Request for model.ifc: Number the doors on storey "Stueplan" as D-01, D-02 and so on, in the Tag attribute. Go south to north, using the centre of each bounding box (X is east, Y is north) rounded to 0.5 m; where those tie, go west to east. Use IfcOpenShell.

First a look at what the model holds.

```python
import ifcopenshell
import ifcopenshell.util.element
import ifcopenshell.util.placement

model = ifcopenshell.open("model.ifc")
print(model.schema)
storey = next(s for s in model.by_type("IfcBuildingStorey") if s.Name == "Stueplan")
doors = [e for e in ifcopenshell.util.element.get_decomposition(storey) if e.is_a("IfcDoor")]
for e in sorted(doors, key=lambda e: e.id()):
    origin = ifcopenshell.util.placement.get_local_placement(e.ObjectPlacement)[:3, 3]
    print(e.id(), e.Tag, e.Name, origin.round(2) + 0.0, sep=" | ")
```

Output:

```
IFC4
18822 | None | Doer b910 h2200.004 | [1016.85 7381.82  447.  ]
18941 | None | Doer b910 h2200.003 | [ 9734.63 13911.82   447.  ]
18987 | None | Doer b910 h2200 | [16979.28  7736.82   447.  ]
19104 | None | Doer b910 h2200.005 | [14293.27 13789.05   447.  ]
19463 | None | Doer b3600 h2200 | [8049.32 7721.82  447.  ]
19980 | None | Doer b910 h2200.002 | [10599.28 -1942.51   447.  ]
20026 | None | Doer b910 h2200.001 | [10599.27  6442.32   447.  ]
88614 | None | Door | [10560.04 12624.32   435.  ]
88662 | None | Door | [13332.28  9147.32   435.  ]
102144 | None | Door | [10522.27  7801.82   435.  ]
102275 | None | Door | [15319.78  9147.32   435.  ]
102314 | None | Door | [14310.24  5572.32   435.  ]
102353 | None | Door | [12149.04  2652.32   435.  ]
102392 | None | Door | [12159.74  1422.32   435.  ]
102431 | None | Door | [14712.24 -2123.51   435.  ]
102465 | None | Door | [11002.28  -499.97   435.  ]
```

```python
import ifcopenshell
import ifcopenshell.geom
import ifcopenshell.util.element
import ifcopenshell.util.shape

model = ifcopenshell.open("model.ifc")
settings = ifcopenshell.geom.settings()
settings.set("use-world-coords", True)


def centre(element):
    shape = ifcopenshell.geom.create_shape(settings, element)
    return ifcopenshell.util.shape.get_bbox_centroid(shape.geometry)


storey = next(s for s in model.by_type("IfcBuildingStorey") if s.Name == "Stueplan")
doors = [e for e in ifcopenshell.util.element.get_decomposition(storey) if e.is_a("IfcDoor")]

# Insertion points can sit at a corner or the storey origin, so sort by the geometry (in metres).
centres = {e: centre(e) for e in doors}
doors.sort(key=lambda e: (round(centres[e][1] / 0.5), centres[e][0]))

for i, e in enumerate(doors, start=1):
    number = f"D-{i:02d}"
    e.Tag = number
    print(e.id(), number)

model.write("model_rev.ifc")
```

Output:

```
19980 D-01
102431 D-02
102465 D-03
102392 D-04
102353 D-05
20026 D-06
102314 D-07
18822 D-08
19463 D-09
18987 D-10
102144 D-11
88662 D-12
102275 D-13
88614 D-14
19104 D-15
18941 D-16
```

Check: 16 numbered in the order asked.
